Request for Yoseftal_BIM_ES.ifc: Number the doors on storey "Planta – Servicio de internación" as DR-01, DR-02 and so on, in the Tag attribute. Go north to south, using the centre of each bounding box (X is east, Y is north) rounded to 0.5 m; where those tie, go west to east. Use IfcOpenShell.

First a look at what the model holds.

```python
import ifcopenshell
import ifcopenshell.util.element
import ifcopenshell.util.placement

model = ifcopenshell.open("Yoseftal_BIM_ES.ifc")
print(model.schema)
storey = next(s for s in model.by_type("IfcBuildingStorey") if s.Name == "Planta – Servicio de internación")
doors = [e for e in ifcopenshell.util.element.get_decomposition(storey) if e.is_a("IfcDoor")]
for e in sorted(doors, key=lambda e: e.id()):
    origin = ifcopenshell.util.placement.get_local_placement(e.ObjectPlacement)[:3, 3]
    print(e.id(), e.Tag, e.Name, origin.round(2) + 0.0, sep=" | ")
```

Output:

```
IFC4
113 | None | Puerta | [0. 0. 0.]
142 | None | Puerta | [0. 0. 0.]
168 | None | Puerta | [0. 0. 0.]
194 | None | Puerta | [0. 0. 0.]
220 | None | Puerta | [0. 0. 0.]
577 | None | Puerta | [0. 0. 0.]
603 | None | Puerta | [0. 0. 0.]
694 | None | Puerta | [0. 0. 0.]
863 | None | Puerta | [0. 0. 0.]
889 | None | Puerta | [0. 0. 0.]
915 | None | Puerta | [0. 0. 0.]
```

```python
import ifcopenshell
import ifcopenshell.geom
import ifcopenshell.util.element
import ifcopenshell.util.shape

model = ifcopenshell.open("Yoseftal_BIM_ES.ifc")
settings = ifcopenshell.geom.settings()
settings.set("use-world-coords", True)


def centre(element):
    shape = ifcopenshell.geom.create_shape(settings, element)
    return ifcopenshell.util.shape.get_bbox_centroid(shape.geometry)


storey = next(s for s in model.by_type("IfcBuildingStorey") if s.Name == "Planta – Servicio de internación")
doors = [e for e in ifcopenshell.util.element.get_decomposition(storey) if e.is_a("IfcDoor")]

# Insertion points can sit at a corner or the storey origin, so sort by the geometry (in metres).
centres = {e: centre(e) for e in doors}
doors.sort(key=lambda e: (-round(centres[e][1] / 0.5), centres[e][0]))

for i, e in enumerate(doors, start=1):
    number = f"DR-{i:02d}"
    e.Tag = number
    print(e.id(), number)

model.write("Yoseftal_BIM_ES_edited.ifc")
```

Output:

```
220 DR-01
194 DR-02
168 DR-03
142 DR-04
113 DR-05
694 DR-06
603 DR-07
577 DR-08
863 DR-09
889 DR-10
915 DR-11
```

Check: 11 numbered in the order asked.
